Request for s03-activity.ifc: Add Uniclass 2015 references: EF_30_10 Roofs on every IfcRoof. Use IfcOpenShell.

First a look at what the model holds.

```python
import ifcopenshell

model = ifcopenshell.open("s03-activity.ifc")
print(model.schema)
print("classifications:", [c.Name for c in model.by_type("IfcClassification")])
for ifc_class in ("IfcDoor", "IfcRoof", "IfcStair", "IfcWall", "IfcWindow"):
    print(ifc_class, len(model.by_type(ifc_class)))
```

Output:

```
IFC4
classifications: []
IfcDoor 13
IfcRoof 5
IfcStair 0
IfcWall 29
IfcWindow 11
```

```python
import ifcopenshell
import ifcopenshell.api.classification

model = ifcopenshell.open("s03-activity.ifc")

system = ifcopenshell.api.classification.add_classification(model, classification="Uniclass 2015")

codes = {
    "IfcRoof": ("EF_30_10", "Roofs"),
}
for ifc_class, (code, name) in codes.items():
    products = model.by_type(ifc_class)
    ifcopenshell.api.classification.add_reference(
        model, products=products, classification=system, identification=code, name=name
    )
    print(code, len(products))

model.write("s03-activity_v2.ifc")
```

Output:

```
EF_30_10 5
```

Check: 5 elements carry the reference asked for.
